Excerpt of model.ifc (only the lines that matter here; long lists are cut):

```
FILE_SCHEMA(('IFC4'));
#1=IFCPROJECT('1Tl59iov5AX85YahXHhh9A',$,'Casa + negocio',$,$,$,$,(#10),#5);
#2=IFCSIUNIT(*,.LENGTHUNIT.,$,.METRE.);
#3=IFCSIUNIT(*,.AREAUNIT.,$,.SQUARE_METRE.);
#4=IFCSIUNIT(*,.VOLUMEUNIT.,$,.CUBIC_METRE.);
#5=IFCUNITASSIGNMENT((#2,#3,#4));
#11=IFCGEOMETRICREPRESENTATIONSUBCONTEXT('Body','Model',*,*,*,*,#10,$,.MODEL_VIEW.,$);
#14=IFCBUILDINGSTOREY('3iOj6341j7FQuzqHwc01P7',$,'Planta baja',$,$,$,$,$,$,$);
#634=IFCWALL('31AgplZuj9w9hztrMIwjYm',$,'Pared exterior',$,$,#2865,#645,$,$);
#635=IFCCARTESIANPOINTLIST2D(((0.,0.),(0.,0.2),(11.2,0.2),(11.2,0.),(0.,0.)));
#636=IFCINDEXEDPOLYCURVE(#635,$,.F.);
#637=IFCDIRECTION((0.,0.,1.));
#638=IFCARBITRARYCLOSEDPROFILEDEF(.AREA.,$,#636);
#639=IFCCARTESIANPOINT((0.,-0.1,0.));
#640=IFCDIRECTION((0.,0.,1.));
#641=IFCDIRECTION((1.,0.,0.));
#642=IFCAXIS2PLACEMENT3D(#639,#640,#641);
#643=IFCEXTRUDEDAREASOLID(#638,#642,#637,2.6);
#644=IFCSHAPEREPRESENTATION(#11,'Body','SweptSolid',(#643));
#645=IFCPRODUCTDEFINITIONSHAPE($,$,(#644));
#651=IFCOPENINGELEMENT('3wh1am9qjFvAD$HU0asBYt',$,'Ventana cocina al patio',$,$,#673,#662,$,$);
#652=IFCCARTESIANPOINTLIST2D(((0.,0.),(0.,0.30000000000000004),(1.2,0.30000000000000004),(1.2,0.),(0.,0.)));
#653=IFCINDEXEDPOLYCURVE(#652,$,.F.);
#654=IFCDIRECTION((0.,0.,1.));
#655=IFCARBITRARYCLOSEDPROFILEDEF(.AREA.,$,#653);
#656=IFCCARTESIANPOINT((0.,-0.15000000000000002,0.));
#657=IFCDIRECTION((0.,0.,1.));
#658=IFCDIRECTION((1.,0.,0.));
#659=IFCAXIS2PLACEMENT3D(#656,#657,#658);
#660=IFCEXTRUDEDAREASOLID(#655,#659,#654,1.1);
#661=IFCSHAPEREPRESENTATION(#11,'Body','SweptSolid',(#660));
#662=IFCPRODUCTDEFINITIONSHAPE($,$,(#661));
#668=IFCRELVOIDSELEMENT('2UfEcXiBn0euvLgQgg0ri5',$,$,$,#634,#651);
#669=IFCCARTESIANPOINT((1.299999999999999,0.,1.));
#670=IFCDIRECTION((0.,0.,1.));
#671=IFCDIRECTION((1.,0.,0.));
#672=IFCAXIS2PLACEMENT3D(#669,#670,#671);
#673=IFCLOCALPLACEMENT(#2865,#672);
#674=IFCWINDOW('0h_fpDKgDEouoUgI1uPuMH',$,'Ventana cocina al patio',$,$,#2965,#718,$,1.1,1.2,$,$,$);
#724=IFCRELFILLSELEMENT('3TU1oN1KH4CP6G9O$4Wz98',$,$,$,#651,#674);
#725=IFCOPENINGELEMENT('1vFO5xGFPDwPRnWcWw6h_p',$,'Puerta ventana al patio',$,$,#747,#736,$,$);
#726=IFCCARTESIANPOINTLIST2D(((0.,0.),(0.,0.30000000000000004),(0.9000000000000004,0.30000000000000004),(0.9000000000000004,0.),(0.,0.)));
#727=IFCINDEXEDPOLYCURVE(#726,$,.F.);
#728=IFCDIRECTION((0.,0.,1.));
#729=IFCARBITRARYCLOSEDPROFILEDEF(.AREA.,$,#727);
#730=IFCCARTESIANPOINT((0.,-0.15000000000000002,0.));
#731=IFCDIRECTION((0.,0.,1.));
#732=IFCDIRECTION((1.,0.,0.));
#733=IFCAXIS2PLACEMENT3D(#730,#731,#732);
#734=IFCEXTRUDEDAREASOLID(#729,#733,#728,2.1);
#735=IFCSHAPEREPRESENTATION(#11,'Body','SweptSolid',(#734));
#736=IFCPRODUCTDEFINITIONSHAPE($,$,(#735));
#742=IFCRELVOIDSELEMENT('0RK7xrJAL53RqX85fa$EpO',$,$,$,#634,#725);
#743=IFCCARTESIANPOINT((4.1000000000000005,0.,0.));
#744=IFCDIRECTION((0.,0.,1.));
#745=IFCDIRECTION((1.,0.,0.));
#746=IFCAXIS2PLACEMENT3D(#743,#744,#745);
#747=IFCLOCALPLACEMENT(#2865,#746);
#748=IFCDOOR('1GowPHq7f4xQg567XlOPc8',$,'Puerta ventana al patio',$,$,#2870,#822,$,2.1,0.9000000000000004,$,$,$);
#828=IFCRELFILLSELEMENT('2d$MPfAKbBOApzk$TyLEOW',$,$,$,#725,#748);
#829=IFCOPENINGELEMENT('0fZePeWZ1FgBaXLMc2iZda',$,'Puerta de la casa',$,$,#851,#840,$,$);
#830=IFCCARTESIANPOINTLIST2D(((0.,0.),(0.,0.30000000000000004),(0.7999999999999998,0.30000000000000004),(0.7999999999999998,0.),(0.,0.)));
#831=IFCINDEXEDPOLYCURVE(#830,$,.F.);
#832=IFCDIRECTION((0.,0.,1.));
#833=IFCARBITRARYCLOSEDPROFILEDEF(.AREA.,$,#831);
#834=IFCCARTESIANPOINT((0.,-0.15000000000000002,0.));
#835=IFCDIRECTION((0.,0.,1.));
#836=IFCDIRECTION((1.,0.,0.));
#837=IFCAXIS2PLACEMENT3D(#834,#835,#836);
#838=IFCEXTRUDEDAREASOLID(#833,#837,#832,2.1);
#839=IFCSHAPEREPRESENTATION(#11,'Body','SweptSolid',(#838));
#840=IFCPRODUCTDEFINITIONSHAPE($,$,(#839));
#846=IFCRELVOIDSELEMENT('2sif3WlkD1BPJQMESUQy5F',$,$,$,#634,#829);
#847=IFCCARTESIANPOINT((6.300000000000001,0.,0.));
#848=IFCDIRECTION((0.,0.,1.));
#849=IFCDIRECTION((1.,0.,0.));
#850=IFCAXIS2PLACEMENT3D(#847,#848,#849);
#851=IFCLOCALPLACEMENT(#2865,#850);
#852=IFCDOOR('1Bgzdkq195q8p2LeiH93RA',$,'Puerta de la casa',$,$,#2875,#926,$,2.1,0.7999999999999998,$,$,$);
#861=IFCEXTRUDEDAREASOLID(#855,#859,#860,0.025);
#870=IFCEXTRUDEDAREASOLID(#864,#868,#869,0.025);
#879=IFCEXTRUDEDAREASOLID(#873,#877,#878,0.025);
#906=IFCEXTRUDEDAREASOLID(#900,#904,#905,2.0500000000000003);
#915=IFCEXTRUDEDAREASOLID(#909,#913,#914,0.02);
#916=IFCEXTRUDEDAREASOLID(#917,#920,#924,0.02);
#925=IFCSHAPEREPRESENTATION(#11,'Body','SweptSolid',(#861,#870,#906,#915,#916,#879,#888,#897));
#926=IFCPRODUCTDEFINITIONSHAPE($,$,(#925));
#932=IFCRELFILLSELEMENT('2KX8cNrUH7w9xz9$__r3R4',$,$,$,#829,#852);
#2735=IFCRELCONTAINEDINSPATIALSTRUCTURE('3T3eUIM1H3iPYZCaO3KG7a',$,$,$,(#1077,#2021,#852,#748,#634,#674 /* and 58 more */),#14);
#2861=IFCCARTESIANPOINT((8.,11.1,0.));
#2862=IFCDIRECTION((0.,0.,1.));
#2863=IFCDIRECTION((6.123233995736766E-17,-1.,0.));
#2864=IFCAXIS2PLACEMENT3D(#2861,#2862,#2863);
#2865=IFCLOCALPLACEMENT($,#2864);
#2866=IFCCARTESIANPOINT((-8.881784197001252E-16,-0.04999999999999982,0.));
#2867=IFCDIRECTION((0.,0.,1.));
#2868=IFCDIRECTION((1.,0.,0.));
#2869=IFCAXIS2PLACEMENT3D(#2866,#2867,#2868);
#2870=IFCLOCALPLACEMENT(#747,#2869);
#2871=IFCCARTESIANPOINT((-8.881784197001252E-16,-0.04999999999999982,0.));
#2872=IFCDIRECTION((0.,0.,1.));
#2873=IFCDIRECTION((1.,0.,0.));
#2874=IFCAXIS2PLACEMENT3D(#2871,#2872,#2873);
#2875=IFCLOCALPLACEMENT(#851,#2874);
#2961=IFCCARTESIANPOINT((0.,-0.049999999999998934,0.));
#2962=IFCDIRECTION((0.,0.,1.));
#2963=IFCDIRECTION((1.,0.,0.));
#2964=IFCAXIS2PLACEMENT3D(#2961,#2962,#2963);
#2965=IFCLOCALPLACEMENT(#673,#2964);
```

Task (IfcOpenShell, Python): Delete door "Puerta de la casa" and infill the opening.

```python
import ifcopenshell
import ifcopenshell.api.feature
import ifcopenshell.api.root
import ifcopenshell.geom
import ifcopenshell.util.shape

model = ifcopenshell.open("model.ifc")
settings = ifcopenshell.geom.settings()


def volume(element):
    """Net volume in cubic metres, openings subtracted."""
    shape = ifcopenshell.geom.create_shape(settings, element)
    return ifcopenshell.util.shape.get_volume(shape.geometry)


door = model.by_guid("1Bgzdkq195q8p2LeiH93RA")
opening = door.FillsVoids[0].RelatingOpeningElement
wall = opening.VoidsElements[0].RelatingBuildingElement
before = volume(wall)

ifcopenshell.api.root.remove_product(model, product=door)
ifcopenshell.api.feature.remove_feature(model, feature=opening)

after = volume(wall)

print(f"wall volume {before:.3f} -> {after:.3f} m3")

model.write("model_updated.ifc")
```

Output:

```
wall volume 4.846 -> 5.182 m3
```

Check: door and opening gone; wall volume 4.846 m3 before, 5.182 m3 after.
